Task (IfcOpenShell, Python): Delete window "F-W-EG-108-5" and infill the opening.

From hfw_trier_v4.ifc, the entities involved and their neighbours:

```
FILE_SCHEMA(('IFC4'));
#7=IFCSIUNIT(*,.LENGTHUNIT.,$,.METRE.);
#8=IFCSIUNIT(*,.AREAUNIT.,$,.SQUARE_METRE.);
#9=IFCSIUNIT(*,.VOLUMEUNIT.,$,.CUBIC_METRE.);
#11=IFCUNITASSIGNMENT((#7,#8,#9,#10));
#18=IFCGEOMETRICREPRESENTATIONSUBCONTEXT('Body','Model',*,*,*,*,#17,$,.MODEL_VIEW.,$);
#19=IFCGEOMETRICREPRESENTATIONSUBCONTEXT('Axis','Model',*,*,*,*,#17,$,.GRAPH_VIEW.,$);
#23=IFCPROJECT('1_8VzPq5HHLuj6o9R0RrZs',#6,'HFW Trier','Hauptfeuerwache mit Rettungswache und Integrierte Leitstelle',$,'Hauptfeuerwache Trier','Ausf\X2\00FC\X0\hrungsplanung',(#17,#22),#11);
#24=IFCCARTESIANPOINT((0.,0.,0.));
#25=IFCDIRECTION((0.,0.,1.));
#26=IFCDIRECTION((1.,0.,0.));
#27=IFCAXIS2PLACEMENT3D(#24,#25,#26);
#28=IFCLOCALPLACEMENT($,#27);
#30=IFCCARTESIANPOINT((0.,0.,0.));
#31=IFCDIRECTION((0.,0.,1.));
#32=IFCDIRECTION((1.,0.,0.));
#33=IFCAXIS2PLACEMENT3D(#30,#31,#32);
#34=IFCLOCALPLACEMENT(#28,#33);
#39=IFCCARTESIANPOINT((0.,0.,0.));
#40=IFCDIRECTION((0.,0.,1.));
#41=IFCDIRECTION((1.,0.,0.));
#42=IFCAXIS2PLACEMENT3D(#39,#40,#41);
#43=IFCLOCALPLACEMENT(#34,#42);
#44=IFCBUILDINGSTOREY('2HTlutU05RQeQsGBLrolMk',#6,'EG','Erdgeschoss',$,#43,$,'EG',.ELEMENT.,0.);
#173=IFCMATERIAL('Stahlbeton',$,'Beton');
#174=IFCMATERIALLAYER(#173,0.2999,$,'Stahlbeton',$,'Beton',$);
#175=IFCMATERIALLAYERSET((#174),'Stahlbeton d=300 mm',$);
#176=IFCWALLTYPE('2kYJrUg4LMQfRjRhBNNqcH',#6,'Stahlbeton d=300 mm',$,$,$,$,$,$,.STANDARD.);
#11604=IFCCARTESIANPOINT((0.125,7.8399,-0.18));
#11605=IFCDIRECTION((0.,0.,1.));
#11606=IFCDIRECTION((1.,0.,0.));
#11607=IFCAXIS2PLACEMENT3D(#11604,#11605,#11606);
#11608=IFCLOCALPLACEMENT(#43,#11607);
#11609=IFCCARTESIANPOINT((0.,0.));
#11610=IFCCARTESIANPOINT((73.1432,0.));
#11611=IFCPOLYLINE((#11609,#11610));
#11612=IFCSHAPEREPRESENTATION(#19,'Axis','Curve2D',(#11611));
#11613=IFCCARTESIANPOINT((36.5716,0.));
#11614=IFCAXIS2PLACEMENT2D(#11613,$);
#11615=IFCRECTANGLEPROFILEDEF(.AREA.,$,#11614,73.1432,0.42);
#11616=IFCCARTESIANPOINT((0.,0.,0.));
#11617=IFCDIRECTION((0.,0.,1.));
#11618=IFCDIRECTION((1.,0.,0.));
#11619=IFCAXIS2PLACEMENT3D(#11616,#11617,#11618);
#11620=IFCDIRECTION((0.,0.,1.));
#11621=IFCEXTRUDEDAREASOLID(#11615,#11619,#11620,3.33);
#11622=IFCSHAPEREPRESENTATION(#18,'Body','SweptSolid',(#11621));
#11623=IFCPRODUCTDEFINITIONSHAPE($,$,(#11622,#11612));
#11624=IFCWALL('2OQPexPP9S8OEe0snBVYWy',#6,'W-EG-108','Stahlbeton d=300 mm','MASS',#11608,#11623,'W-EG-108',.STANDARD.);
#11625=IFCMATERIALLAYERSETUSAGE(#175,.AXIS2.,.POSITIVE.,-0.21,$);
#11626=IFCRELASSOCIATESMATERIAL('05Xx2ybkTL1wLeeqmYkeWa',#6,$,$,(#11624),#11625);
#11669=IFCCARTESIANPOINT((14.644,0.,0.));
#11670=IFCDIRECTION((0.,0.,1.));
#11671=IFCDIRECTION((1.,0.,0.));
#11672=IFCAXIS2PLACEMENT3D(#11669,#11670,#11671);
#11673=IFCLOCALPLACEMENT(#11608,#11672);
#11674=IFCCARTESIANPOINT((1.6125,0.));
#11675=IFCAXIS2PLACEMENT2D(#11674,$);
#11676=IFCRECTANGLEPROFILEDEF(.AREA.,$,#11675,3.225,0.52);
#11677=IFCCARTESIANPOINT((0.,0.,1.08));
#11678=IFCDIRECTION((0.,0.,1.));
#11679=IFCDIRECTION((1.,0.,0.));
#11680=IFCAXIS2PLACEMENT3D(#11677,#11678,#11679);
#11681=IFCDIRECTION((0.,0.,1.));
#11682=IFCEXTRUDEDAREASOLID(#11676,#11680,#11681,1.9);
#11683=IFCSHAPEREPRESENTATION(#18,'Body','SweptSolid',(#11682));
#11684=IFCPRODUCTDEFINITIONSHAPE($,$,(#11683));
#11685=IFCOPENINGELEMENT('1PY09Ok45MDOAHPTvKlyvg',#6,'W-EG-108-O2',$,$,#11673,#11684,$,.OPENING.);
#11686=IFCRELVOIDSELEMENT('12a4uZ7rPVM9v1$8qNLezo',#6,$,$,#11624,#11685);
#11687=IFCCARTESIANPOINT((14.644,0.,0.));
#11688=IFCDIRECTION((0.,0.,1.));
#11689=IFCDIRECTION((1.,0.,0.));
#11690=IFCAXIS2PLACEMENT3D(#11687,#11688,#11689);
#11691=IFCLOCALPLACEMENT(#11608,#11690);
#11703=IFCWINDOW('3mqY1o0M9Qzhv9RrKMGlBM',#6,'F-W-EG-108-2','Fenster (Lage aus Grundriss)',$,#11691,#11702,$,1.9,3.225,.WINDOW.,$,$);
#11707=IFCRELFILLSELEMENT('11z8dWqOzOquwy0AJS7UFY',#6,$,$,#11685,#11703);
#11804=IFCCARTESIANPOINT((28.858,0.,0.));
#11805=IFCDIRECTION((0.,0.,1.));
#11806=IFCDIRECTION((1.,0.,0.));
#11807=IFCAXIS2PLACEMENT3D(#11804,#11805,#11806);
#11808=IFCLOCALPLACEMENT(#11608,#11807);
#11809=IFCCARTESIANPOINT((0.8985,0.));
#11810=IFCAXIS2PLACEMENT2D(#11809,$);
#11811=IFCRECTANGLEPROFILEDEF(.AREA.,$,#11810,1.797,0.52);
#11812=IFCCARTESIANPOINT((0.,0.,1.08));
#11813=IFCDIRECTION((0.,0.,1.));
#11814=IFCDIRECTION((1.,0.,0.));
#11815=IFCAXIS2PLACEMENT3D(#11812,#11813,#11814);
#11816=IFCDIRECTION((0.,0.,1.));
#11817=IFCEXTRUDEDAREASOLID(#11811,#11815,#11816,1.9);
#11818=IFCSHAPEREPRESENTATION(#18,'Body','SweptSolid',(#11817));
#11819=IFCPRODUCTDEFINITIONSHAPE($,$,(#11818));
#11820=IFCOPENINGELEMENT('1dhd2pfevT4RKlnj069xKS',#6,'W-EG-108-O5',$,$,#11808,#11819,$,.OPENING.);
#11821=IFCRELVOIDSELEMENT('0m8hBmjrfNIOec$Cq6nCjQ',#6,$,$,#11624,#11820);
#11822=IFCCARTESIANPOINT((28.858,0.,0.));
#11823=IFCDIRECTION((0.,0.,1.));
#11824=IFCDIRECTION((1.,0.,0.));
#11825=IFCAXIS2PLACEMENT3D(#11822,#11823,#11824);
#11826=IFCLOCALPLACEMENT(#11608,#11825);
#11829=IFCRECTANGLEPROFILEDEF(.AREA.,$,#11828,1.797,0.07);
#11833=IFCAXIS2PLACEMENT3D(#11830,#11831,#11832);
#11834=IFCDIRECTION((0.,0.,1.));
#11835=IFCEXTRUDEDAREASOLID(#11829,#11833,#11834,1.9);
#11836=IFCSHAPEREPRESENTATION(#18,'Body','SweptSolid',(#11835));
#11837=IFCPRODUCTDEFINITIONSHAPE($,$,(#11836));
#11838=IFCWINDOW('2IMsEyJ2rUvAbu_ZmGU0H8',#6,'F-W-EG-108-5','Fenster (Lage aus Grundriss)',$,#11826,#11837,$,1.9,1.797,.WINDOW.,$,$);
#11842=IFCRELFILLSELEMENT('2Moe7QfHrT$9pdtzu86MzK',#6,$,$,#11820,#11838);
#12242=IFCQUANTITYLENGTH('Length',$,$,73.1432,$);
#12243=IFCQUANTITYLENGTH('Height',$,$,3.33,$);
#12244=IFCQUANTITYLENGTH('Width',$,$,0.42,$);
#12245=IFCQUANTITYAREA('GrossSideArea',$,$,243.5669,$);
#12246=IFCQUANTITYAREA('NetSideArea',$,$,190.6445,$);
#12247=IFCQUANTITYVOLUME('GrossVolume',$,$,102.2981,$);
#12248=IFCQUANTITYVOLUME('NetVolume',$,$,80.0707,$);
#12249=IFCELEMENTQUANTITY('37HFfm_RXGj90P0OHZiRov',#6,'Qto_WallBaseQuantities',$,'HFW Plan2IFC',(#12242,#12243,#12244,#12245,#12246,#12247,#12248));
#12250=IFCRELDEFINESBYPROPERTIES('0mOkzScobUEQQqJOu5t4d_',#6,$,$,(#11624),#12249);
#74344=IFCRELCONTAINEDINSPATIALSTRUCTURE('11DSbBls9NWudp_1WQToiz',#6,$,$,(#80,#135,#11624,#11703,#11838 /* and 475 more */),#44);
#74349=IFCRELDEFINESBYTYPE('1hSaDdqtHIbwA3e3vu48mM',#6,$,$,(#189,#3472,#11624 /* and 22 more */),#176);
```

```python
import ifcopenshell
import ifcopenshell.api.feature
import ifcopenshell.api.pset
import ifcopenshell.api.root
import ifcopenshell.geom
import ifcopenshell.util.element
import ifcopenshell.util.shape
import ifcopenshell.util.unit

model = ifcopenshell.open("hfw_trier_v4.ifc")
area_scale = ifcopenshell.util.unit.calculate_unit_scale(model, "AREAUNIT")
volume_scale = ifcopenshell.util.unit.calculate_unit_scale(model, "VOLUMEUNIT")
settings = ifcopenshell.geom.settings()


def volume(element):
    """Net volume in cubic metres, openings subtracted."""
    shape = ifcopenshell.geom.create_shape(settings, element)
    return ifcopenshell.util.shape.get_volume(shape.geometry)


window = model.by_id(11838)
opening = window.FillsVoids[0].RelatingOpeningElement
wall = opening.VoidsElements[0].RelatingBuildingElement
before = volume(wall)

ifcopenshell.api.root.remove_product(model, product=window)
ifcopenshell.api.feature.remove_feature(model, feature=opening)

after = volume(wall)
thickness = 0.42  # wall thickness in metres

# Update the wall's stored quantities.
qto = model.by_id(ifcopenshell.util.element.get_pset(wall, "Qto_WallBaseQuantities", should_inherit=False)["id"])
ifcopenshell.api.pset.edit_qto(model, qto=qto, properties={
    "NetSideArea": after / thickness / area_scale,
    "NetVolume": after / volume_scale,
})

print(f"wall volume {before:.3f} -> {after:.3f} m3")

model.write("hfw_trier_v4_v2.ifc")
```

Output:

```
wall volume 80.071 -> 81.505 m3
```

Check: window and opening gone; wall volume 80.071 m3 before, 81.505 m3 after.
